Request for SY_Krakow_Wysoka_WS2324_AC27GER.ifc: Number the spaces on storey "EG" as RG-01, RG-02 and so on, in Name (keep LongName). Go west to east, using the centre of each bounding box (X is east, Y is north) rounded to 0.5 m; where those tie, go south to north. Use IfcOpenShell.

First a look at what the model holds.

```python
import ifcopenshell
import ifcopenshell.util.element
import ifcopenshell.util.placement

model = ifcopenshell.open("SY_Krakow_Wysoka_WS2324_AC27GER.ifc")
print(model.schema)
storey = next(s for s in model.by_type("IfcBuildingStorey") if s.Name == "EG")
spaces = [e for e in ifcopenshell.util.element.get_decomposition(storey) if e.is_a("IfcSpace")]
for e in sorted(spaces, key=lambda e: e.id()):
    origin = ifcopenshell.util.placement.get_local_placement(e.ObjectPlacement)[:3, 3]
    print(e.id(), e.Name, e.LongName, origin.round(2) + 0.0, sep=" | ")
```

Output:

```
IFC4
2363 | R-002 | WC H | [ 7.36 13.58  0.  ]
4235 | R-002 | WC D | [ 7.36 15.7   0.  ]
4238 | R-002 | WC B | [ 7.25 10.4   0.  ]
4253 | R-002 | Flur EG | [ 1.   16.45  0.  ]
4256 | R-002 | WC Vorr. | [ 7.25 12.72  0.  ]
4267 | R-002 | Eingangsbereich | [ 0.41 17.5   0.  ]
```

```python
import ifcopenshell
import ifcopenshell.geom
import ifcopenshell.util.element
import ifcopenshell.util.shape

model = ifcopenshell.open("SY_Krakow_Wysoka_WS2324_AC27GER.ifc")
settings = ifcopenshell.geom.settings()
settings.set("use-world-coords", True)


def centre(element):
    shape = ifcopenshell.geom.create_shape(settings, element)
    return ifcopenshell.util.shape.get_bbox_centroid(shape.geometry)


storey = next(s for s in model.by_type("IfcBuildingStorey") if s.Name == "EG")
spaces = [e for e in ifcopenshell.util.element.get_decomposition(storey) if e.is_a("IfcSpace")]

# Insertion points can sit at a corner or the storey origin, so sort by the geometry (in metres).
centres = {e: centre(e) for e in spaces}
spaces.sort(key=lambda e: (round(centres[e][0] / 0.5), centres[e][1]))

for i, e in enumerate(spaces, start=1):
    number = f"RG-{i:02d}"
    e.Name = number
    print(e.id(), number)

model.write("SY_Krakow_Wysoka_WS2324_AC27GER_edited.ifc")
```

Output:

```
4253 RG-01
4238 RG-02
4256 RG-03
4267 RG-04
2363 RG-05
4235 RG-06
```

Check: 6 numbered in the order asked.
